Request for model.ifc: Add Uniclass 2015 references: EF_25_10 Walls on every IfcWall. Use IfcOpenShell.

First a look at what the model holds.

```python
import ifcopenshell

model = ifcopenshell.open("model.ifc")
print(model.schema)
print("classifications:", [c.Name for c in model.by_type("IfcClassification")])
for ifc_class in ("IfcDoor", "IfcRoof", "IfcStair", "IfcWall", "IfcWindow"):
    print(ifc_class, len(model.by_type(ifc_class)))
```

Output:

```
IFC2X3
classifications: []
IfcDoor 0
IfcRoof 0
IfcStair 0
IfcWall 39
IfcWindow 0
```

```python
import ifcopenshell
import ifcopenshell.api.classification

model = ifcopenshell.open("model.ifc")

# IFC2X3 requires Source and Edition and has no link from the project to the system.
system = model.create_entity("IfcClassification", Source="NBS", Edition="2015", Name="Uniclass 2015")

codes = {
    "IfcWall": ("EF_25_10", "Walls"),
}
for ifc_class, (code, name) in codes.items():
    products = model.by_type(ifc_class)
    ifcopenshell.api.classification.add_reference(
        model, products=products, classification=system, identification=code, name=name
    )
    print(code, len(products))

model.write("model_rev.ifc")
```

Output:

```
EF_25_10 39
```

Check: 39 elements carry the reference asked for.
